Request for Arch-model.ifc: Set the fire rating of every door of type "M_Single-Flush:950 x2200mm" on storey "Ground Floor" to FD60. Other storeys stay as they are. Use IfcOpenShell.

First a look at what the model holds.

```python
import ifcopenshell
import ifcopenshell.util.element

model = ifcopenshell.open("Arch-model.ifc")
print(model.schema)
storey = next(s for s in model.by_type("IfcBuildingStorey") if s.Name == "Ground Floor")
doors = [e for e in ifcopenshell.util.element.get_decomposition(storey) if e.is_a("IfcDoor")]
seen = {}
for e in doors:
    element_type = ifcopenshell.util.element.get_type(e)
    key = (element_type.Name if element_type != e and element_type else None, ifcopenshell.util.element.get_pset(e, "Pset_DoorCommon", "FireRating"))
    seen[key] = seen.get(key, 0) + 1
for (name, value), count in sorted(seen.items(), key=str):
    print(count, "x", name, "|", value)
```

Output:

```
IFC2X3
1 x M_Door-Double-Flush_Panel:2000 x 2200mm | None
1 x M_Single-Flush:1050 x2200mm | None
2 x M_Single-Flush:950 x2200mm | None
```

```python
import ifcopenshell
import ifcopenshell.api.pset
import ifcopenshell.util.element

model = ifcopenshell.open("Arch-model.ifc")

storey = next(s for s in model.by_type("IfcBuildingStorey") if s.Name == "Ground Floor")
doors = [e for e in ifcopenshell.util.element.get_decomposition(storey) if e.is_a("IfcDoor")]

count = 0
for e in doors:
    element_type = ifcopenshell.util.element.get_type(e)
    if element_type in (None, e) or element_type.Name != "M_Single-Flush:950 x2200mm":
        continue
    # add_pset returns the element's existing set when there is one.
    pset = ifcopenshell.api.pset.add_pset(model, product=e, name="Pset_DoorCommon")
    ifcopenshell.api.pset.edit_pset(model, pset=pset, properties={"FireRating": "FD60"})
    count += 1

print(count, "doors updated")

model.write("Arch-model_updated.ifc")
```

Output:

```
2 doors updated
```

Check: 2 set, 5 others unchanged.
